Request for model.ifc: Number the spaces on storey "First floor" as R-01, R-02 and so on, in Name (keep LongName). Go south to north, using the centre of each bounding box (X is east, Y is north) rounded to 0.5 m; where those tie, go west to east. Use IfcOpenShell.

First a look at what the model holds.

```python
import ifcopenshell
import ifcopenshell.util.element
import ifcopenshell.util.placement

model = ifcopenshell.open("model.ifc")
print(model.schema)
storey = next(s for s in model.by_type("IfcBuildingStorey") if s.Name == "First floor")
spaces = [e for e in ifcopenshell.util.element.get_decomposition(storey) if e.is_a("IfcSpace")]
for e in sorted(spaces, key=lambda e: e.id()):
    origin = ifcopenshell.util.placement.get_local_placement(e.ObjectPlacement)[:3, 3]
    print(e.id(), e.Name, e.LongName, origin.round(2) + 0.0, sep=" | ")
```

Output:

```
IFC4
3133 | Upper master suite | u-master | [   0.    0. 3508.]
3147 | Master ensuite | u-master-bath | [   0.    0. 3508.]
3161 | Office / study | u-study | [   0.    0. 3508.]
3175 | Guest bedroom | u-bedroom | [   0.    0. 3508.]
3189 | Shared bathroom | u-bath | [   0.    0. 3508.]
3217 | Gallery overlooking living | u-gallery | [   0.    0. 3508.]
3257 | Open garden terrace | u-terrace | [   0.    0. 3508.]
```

```python
import ifcopenshell
import ifcopenshell.geom
import ifcopenshell.util.element
import ifcopenshell.util.shape

model = ifcopenshell.open("model.ifc")
settings = ifcopenshell.geom.settings()
settings.set("use-world-coords", True)


def centre(element):
    shape = ifcopenshell.geom.create_shape(settings, element)
    return ifcopenshell.util.shape.get_bbox_centroid(shape.geometry)


storey = next(s for s in model.by_type("IfcBuildingStorey") if s.Name == "First floor")
spaces = [e for e in ifcopenshell.util.element.get_decomposition(storey) if e.is_a("IfcSpace")]

# Insertion points can sit at a corner or the storey origin, so sort by the geometry (in metres).
centres = {e: centre(e) for e in spaces}
spaces.sort(key=lambda e: (round(centres[e][1] / 0.5), centres[e][0]))

for i, e in enumerate(spaces, start=1):
    number = f"R-{i:02d}"
    e.Name = number
    print(e.id(), number)

model.write("model_rev.ifc")
```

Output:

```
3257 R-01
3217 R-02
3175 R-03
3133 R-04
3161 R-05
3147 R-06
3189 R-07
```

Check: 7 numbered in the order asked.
